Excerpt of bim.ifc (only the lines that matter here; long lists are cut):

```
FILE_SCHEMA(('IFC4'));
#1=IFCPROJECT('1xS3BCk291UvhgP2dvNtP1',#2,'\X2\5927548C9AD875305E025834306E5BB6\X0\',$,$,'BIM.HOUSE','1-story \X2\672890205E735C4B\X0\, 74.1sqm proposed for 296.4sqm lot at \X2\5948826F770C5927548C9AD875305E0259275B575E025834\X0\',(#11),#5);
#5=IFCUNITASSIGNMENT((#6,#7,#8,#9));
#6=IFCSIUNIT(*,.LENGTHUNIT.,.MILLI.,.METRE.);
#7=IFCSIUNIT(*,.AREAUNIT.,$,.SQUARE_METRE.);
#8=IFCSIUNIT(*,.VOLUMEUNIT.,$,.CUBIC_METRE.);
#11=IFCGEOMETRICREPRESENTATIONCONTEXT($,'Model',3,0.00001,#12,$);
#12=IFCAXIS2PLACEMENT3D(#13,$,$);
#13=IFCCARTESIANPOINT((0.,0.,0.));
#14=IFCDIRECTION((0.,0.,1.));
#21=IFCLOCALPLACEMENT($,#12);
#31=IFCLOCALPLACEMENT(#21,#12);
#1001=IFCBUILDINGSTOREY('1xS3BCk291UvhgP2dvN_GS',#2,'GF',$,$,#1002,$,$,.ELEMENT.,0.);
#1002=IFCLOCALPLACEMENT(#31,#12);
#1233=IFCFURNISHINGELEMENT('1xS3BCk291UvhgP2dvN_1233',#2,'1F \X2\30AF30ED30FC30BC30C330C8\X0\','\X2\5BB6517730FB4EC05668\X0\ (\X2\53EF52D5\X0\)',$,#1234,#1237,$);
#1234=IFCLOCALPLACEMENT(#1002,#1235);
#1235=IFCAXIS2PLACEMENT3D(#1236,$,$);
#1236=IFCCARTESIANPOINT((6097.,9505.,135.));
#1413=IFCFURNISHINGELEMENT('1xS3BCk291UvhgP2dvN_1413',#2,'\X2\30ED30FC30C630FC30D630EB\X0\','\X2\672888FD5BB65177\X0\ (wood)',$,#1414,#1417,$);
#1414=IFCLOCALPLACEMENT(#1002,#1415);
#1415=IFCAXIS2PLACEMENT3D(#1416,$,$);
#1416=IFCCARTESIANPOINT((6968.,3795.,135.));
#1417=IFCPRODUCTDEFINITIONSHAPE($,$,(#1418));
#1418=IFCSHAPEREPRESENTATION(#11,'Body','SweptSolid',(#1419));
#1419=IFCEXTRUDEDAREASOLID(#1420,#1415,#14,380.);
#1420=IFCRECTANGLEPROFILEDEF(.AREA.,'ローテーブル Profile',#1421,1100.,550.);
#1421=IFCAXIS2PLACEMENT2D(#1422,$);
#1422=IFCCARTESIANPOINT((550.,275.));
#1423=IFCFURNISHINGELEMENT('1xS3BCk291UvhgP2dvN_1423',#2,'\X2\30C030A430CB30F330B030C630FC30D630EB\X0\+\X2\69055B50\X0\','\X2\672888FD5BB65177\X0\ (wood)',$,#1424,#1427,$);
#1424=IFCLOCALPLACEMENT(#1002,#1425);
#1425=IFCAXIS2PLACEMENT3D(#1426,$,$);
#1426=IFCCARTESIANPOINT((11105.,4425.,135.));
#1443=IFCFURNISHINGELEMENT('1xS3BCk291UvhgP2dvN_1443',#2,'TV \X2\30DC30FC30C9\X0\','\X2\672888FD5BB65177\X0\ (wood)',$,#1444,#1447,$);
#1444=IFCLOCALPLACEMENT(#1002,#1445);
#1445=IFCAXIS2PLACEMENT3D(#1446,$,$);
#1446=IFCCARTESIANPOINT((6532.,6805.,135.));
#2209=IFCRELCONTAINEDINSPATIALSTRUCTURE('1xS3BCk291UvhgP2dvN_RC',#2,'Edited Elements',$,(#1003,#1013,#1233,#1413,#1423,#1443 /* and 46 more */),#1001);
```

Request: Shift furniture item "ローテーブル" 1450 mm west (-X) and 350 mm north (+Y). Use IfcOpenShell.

```python
import ifcopenshell
import ifcopenshell.api.geometry
import ifcopenshell.util.placement
import ifcopenshell.util.unit

model = ifcopenshell.open("bim.ifc")
unit_scale = ifcopenshell.util.unit.calculate_unit_scale(model)

item = model.by_id(1413)
matrix = ifcopenshell.util.placement.get_local_placement(item.ObjectPlacement)
matrix[0, 3] -= 1.45 / unit_scale
matrix[1, 3] += 0.35 / unit_scale
ifcopenshell.api.geometry.edit_object_placement(model, product=item, matrix=matrix, is_si=False)

print(ifcopenshell.util.placement.get_local_placement(item.ObjectPlacement).round(3) + 0.0)

model.write("bim-out.ifc")
```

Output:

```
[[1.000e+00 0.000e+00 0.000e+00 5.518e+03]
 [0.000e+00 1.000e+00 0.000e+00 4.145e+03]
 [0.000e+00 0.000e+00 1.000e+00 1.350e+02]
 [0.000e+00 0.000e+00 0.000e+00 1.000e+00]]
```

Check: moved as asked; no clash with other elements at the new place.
